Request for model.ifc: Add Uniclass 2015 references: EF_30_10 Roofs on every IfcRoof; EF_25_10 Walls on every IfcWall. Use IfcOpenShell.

First a look at what the model holds.

```python
import ifcopenshell

model = ifcopenshell.open("model.ifc")
print(model.schema)
print("classifications:", [c.Name for c in model.by_type("IfcClassification")])
for ifc_class in ("IfcDoor", "IfcRoof", "IfcStair", "IfcWall", "IfcWindow"):
    print(ifc_class, len(model.by_type(ifc_class)))
```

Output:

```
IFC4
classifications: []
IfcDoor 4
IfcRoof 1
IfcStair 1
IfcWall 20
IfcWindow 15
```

```python
import ifcopenshell
import ifcopenshell.api.classification

model = ifcopenshell.open("model.ifc")

system = ifcopenshell.api.classification.add_classification(model, classification="Uniclass 2015")

codes = {
    "IfcRoof": ("EF_30_10", "Roofs"),
    "IfcWall": ("EF_25_10", "Walls"),
}
for ifc_class, (code, name) in codes.items():
    products = model.by_type(ifc_class)
    ifcopenshell.api.classification.add_reference(
        model, products=products, classification=system, identification=code, name=name
    )
    print(code, len(products))

model.write("model_updated.ifc")
```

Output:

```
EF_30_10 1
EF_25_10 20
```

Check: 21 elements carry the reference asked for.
